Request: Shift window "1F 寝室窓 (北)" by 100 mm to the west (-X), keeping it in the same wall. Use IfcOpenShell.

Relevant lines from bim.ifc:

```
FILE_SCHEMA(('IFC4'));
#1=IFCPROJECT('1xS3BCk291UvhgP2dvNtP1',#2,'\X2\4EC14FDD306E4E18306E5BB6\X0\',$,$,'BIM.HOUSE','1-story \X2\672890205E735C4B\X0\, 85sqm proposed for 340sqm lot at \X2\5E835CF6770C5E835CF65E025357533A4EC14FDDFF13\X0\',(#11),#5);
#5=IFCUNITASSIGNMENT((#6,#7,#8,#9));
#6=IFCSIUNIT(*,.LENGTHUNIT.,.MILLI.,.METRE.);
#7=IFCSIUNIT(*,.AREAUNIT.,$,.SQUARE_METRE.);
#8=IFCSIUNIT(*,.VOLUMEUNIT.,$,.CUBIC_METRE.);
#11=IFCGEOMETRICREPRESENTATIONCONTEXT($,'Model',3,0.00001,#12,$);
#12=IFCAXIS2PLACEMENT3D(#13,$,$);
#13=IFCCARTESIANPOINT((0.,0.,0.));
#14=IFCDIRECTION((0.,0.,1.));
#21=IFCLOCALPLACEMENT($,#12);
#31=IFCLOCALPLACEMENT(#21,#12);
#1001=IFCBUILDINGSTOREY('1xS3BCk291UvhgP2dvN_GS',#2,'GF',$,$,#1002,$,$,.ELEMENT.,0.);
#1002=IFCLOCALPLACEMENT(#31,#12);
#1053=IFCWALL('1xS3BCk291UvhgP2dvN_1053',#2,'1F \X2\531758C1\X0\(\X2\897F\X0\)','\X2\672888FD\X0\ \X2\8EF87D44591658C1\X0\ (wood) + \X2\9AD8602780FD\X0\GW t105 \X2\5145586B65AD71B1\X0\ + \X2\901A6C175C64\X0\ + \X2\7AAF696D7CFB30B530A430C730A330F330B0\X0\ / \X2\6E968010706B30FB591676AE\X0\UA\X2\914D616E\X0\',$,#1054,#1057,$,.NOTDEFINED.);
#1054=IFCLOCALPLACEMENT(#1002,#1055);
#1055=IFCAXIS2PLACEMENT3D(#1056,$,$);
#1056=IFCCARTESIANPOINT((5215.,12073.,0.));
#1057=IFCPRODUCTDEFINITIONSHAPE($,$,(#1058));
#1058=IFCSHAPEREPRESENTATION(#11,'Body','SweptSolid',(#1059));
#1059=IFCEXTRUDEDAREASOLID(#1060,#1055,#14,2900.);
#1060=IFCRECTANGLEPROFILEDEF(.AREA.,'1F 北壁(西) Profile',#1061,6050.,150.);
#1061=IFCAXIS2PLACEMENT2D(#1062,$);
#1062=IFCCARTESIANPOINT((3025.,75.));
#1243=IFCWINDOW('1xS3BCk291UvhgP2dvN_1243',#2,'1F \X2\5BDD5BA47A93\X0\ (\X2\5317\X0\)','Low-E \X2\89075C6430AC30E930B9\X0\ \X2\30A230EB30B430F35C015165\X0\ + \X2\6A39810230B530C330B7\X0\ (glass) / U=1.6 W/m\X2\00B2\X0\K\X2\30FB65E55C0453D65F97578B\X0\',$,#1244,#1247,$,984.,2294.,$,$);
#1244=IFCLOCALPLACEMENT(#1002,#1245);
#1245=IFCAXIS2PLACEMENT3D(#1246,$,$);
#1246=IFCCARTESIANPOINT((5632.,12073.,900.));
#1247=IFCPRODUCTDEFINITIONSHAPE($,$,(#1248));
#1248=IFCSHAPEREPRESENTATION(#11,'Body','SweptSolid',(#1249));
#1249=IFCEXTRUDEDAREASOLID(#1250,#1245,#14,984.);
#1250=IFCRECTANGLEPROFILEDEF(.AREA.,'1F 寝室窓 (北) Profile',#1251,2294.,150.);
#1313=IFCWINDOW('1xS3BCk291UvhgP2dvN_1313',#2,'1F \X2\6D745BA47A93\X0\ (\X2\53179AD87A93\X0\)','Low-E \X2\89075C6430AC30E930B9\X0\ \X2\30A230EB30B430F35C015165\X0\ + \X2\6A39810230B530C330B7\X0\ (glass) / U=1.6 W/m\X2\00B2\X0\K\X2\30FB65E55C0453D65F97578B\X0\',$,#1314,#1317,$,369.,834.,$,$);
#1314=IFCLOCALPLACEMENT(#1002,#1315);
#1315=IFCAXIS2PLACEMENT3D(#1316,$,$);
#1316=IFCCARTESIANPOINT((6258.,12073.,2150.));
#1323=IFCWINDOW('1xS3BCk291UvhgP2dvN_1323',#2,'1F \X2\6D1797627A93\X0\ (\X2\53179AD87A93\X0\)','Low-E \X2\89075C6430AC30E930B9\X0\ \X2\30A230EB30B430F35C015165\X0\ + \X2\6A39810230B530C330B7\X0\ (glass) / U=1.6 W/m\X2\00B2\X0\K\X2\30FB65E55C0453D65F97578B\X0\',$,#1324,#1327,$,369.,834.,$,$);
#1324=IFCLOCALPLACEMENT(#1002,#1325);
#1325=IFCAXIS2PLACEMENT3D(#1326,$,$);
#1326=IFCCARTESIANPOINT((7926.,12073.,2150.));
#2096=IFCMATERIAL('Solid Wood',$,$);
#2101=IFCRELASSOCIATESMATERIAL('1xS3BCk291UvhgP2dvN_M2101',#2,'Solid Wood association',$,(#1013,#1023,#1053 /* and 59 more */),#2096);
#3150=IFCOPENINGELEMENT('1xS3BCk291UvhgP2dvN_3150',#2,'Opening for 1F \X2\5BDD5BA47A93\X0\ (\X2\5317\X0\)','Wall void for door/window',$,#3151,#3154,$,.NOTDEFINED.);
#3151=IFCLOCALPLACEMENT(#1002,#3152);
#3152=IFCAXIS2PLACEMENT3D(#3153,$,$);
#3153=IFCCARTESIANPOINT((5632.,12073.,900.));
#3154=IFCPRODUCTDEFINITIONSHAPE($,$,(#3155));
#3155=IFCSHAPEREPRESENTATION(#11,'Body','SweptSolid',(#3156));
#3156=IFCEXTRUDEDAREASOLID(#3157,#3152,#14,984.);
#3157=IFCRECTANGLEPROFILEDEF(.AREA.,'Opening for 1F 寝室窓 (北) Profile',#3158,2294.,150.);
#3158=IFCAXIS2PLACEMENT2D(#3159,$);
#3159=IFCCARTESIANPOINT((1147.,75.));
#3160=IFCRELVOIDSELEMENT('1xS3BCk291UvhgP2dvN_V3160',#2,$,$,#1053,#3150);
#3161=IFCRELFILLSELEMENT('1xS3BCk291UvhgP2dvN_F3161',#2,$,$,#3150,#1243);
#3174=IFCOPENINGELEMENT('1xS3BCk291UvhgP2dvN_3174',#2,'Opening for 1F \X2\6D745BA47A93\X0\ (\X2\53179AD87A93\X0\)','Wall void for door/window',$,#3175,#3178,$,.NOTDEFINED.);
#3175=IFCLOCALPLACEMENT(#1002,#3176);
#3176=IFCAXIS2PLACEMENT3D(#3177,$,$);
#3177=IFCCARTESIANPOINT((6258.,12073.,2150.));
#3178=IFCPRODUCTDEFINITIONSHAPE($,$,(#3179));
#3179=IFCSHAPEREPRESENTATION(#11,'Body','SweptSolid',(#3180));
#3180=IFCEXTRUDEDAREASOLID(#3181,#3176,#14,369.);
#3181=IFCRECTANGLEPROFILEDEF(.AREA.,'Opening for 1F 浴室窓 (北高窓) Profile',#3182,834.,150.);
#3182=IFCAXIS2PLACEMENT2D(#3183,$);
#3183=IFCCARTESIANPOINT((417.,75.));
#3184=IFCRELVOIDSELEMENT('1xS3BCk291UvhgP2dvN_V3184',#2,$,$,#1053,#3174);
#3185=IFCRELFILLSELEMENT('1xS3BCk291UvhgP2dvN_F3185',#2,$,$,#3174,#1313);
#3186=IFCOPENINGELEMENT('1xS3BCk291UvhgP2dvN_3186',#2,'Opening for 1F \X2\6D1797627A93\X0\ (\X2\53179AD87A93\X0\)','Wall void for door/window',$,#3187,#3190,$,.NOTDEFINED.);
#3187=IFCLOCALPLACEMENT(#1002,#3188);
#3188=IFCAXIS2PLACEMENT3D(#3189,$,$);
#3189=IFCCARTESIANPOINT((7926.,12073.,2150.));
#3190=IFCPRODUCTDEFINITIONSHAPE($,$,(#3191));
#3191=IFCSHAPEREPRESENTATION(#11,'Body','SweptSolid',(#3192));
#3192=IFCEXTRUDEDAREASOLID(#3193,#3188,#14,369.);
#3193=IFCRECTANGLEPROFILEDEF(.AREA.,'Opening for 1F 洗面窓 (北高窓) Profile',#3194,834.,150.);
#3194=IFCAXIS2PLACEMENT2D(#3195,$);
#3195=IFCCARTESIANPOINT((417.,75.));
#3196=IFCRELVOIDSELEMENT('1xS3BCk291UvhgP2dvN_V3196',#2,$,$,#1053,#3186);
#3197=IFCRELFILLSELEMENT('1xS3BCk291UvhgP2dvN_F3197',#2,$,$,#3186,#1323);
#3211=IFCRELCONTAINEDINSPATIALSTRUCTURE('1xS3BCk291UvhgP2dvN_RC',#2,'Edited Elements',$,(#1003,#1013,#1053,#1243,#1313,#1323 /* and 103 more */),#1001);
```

```python
import ifcopenshell
import ifcopenshell.api.geometry
import ifcopenshell.util.placement

model = ifcopenshell.open("bim.ifc")

window = model.by_id(1243)
opening = window.FillsVoids[0].RelatingOpeningElement
wall = opening.VoidsElements[0].RelatingBuildingElement

wall_matrix = ifcopenshell.util.placement.get_local_placement(wall.ObjectPlacement)
shift = wall_matrix[:3, 0] * -100.0
before = ifcopenshell.util.placement.get_local_placement(window.ObjectPlacement)[:3, 3].copy()

# The window is not placed relative to its opening, so move both.
for product in (opening, window):
    matrix = ifcopenshell.util.placement.get_local_placement(product.ObjectPlacement)
    matrix[:3, 3] += shift
    ifcopenshell.api.geometry.edit_object_placement(model, product=product, matrix=matrix, is_si=False)

after = ifcopenshell.util.placement.get_local_placement(window.ObjectPlacement)[:3, 3]
print("window moved by", (after - before).round(3) + 0.0)

model.write("bim_updated.ifc")
```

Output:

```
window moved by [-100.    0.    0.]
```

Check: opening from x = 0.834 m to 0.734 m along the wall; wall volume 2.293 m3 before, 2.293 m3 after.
